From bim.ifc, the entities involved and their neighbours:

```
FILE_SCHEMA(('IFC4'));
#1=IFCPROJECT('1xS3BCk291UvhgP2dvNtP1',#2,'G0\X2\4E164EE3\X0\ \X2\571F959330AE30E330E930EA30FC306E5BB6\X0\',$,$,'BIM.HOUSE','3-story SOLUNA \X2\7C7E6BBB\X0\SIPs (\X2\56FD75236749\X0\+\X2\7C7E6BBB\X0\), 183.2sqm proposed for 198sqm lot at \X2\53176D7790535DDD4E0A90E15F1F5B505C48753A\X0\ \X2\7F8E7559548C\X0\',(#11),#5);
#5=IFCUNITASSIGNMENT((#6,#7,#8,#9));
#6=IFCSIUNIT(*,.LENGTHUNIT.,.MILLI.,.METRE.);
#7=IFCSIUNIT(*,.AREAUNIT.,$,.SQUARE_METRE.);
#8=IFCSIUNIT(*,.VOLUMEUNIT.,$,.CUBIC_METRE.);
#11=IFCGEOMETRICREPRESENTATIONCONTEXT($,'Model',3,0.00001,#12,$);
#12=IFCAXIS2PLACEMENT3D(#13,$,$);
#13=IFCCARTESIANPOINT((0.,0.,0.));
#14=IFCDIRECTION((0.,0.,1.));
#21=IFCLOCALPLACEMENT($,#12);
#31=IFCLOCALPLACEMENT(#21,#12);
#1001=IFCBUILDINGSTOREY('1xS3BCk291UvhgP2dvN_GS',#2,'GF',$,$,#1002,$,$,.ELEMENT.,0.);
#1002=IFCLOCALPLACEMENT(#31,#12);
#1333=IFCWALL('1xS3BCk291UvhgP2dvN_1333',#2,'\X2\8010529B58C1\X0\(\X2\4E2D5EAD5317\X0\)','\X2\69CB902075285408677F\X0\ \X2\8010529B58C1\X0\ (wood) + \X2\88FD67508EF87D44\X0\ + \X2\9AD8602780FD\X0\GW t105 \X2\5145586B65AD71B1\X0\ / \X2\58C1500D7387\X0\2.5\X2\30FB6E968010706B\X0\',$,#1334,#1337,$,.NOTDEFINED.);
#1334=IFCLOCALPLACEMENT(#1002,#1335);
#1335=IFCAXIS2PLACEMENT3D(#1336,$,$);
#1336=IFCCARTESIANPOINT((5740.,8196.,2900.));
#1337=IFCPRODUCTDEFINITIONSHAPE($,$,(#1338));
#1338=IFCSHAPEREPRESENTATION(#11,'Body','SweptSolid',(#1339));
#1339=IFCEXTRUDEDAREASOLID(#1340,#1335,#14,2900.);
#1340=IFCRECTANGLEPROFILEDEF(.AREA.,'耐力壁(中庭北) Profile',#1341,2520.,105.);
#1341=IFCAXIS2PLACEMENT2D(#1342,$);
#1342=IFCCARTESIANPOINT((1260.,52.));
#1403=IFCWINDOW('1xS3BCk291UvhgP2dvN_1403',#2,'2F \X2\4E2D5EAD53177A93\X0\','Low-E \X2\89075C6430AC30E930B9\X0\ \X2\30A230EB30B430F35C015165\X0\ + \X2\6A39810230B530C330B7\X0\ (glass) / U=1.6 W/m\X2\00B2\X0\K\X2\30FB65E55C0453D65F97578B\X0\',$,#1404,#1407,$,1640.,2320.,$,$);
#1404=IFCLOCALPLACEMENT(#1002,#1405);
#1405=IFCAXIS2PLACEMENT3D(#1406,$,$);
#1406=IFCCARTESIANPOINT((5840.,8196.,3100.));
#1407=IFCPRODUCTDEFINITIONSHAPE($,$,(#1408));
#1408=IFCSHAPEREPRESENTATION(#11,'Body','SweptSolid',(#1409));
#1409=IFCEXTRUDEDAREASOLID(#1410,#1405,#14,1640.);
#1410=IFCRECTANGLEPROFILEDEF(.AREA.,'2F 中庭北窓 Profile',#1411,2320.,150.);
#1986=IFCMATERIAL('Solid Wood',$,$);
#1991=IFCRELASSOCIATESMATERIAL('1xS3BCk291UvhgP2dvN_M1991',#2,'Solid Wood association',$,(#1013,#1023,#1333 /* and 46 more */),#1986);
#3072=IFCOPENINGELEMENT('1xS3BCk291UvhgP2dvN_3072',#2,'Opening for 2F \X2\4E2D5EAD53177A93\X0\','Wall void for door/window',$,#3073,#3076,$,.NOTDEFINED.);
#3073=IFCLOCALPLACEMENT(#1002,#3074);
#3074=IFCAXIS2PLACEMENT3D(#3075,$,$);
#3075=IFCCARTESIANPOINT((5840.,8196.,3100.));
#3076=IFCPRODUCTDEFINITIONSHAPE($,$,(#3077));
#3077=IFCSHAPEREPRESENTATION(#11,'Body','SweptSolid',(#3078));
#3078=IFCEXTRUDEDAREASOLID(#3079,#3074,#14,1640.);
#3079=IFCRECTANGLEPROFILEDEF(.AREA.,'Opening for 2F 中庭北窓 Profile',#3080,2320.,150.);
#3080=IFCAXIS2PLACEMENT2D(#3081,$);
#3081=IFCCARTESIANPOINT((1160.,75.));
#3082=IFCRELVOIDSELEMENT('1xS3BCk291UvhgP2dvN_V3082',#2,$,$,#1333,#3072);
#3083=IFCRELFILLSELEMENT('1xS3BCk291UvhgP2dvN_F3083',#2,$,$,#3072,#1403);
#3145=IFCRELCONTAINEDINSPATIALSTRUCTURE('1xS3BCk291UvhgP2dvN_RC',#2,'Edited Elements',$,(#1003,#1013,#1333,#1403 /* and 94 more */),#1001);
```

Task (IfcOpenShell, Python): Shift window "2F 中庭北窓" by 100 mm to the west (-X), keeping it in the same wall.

```python
import ifcopenshell
import ifcopenshell.api.geometry
import ifcopenshell.util.placement

model = ifcopenshell.open("bim.ifc")

window = model.by_guid("1xS3BCk291UvhgP2dvN_1403")
opening = window.FillsVoids[0].RelatingOpeningElement
wall = opening.VoidsElements[0].RelatingBuildingElement

wall_matrix = ifcopenshell.util.placement.get_local_placement(wall.ObjectPlacement)
shift = wall_matrix[:3, 0] * -100.0
before = ifcopenshell.util.placement.get_local_placement(window.ObjectPlacement)[:3, 3].copy()

# The window is not placed relative to its opening, so move both.
for product in (opening, window):
    matrix = ifcopenshell.util.placement.get_local_placement(product.ObjectPlacement)
    matrix[:3, 3] += shift
    ifcopenshell.api.geometry.edit_object_placement(model, product=product, matrix=matrix, is_si=False)

after = ifcopenshell.util.placement.get_local_placement(window.ObjectPlacement)[:3, 3]
print("window moved by", (after - before).round(3) + 0.0)

model.write("bim_rev.ifc")
```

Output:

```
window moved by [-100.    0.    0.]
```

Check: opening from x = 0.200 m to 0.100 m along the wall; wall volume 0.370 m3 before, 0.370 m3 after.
